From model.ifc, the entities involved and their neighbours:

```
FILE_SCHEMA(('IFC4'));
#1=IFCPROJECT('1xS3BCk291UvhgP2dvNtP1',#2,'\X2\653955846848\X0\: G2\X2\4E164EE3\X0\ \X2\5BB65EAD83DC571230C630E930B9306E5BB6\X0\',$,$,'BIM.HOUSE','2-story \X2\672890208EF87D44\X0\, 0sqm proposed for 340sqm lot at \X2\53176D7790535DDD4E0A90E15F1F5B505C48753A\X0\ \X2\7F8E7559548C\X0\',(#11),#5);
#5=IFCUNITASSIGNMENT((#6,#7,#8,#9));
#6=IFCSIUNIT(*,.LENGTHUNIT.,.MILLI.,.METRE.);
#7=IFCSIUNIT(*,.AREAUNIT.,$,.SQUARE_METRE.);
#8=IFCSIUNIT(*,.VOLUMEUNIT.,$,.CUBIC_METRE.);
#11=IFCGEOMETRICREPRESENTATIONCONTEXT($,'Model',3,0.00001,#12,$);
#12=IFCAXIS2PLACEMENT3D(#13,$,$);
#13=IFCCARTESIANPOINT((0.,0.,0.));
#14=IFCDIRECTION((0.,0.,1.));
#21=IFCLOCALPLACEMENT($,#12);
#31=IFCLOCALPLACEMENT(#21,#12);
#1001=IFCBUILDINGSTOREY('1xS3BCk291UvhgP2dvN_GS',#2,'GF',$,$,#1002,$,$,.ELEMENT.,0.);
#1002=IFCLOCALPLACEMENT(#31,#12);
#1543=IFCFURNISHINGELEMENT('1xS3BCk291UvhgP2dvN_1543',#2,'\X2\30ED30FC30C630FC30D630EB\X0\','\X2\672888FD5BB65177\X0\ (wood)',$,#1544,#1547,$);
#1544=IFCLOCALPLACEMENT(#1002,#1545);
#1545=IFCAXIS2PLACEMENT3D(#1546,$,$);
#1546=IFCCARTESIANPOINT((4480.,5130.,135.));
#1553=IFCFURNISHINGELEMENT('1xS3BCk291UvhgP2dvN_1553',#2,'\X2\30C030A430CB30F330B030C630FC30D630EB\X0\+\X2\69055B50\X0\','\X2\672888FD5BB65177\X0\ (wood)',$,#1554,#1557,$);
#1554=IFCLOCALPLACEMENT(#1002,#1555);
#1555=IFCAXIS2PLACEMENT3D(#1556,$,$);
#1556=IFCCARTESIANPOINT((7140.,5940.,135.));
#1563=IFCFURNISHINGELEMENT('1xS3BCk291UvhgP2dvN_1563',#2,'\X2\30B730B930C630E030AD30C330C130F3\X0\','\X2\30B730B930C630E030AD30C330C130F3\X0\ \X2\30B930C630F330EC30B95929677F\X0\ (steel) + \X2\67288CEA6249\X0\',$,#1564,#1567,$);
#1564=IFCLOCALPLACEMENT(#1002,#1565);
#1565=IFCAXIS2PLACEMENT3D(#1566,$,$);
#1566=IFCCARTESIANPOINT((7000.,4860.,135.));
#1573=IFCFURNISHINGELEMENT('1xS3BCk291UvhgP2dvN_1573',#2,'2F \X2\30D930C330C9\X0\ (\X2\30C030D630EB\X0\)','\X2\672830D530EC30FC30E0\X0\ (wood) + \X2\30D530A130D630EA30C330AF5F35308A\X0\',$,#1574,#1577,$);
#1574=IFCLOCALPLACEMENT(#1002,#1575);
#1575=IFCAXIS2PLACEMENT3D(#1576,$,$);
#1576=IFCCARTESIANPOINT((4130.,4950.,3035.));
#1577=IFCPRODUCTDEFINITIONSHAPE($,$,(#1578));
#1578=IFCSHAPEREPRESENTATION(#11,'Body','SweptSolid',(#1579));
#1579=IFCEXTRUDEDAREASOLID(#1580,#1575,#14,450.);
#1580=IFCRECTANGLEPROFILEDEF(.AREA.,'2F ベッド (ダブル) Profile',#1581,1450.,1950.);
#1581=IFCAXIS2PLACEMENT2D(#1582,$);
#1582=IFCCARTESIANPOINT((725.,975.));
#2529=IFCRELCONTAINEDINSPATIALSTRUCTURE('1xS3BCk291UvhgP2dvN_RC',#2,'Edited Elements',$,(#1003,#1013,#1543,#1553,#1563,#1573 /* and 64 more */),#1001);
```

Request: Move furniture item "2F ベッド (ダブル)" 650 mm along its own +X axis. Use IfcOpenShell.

```python
import ifcopenshell
import ifcopenshell.api.geometry
import ifcopenshell.util.placement
import ifcopenshell.util.unit

model = ifcopenshell.open("model.ifc")
unit_scale = ifcopenshell.util.unit.calculate_unit_scale(model)

item = model.by_guid("1xS3BCk291UvhgP2dvN_1573")
matrix = ifcopenshell.util.placement.get_local_placement(item.ObjectPlacement)
matrix[:3, 3] += matrix[:3, 0] * 0.65 / unit_scale
ifcopenshell.api.geometry.edit_object_placement(model, product=item, matrix=matrix, is_si=False)

print(ifcopenshell.util.placement.get_local_placement(item.ObjectPlacement).round(3) + 0.0)

model.write("model-out.ifc")
```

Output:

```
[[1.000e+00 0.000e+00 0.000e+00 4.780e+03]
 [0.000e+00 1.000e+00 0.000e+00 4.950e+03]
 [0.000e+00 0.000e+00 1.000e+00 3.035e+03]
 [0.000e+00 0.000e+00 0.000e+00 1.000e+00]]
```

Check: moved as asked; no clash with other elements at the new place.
